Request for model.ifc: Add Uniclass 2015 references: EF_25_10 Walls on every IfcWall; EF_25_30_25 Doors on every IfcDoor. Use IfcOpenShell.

First a look at what the model holds.

```python
import ifcopenshell

model = ifcopenshell.open("model.ifc")
print(model.schema)
print("classifications:", [c.Name for c in model.by_type("IfcClassification")])
for ifc_class in ("IfcDoor", "IfcRoof", "IfcStair", "IfcWall", "IfcWindow"):
    print(ifc_class, len(model.by_type(ifc_class)))
```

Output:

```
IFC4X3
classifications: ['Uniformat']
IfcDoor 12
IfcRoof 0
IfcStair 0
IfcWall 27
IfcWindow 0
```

```python
import ifcopenshell
import ifcopenshell.api.classification

model = ifcopenshell.open("model.ifc")

system = ifcopenshell.api.classification.add_classification(model, classification="Uniclass 2015")

codes = {
    "IfcWall": ("EF_25_10", "Walls"),
    "IfcDoor": ("EF_25_30_25", "Doors"),
}
for ifc_class, (code, name) in codes.items():
    products = model.by_type(ifc_class)
    ifcopenshell.api.classification.add_reference(
        model, products=products, classification=system, identification=code, name=name
    )
    print(code, len(products))

model.write("model_edited.ifc")
```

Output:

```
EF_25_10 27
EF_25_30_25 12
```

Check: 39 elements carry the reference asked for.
